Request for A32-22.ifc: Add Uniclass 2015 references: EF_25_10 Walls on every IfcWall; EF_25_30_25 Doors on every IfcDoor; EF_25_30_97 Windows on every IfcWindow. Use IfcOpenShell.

First a look at what the model holds.

```python
import ifcopenshell

model = ifcopenshell.open("A32-22.ifc")
print(model.schema)
print("classifications:", [c.Name for c in model.by_type("IfcClassification")])
for ifc_class in ("IfcDoor", "IfcRoof", "IfcStair", "IfcWall", "IfcWindow"):
    print(ifc_class, len(model.by_type(ifc_class)))
```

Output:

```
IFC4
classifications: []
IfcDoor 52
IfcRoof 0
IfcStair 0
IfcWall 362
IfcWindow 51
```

```python
import ifcopenshell
import ifcopenshell.api.classification

model = ifcopenshell.open("A32-22.ifc")

system = ifcopenshell.api.classification.add_classification(model, classification="Uniclass 2015")

codes = {
    "IfcWall": ("EF_25_10", "Walls"),
    "IfcDoor": ("EF_25_30_25", "Doors"),
    "IfcWindow": ("EF_25_30_97", "Windows"),
}
for ifc_class, (code, name) in codes.items():
    products = model.by_type(ifc_class)
    ifcopenshell.api.classification.add_reference(
        model, products=products, classification=system, identification=code, name=name
    )
    print(code, len(products))

model.write("A32-22_v2.ifc")
```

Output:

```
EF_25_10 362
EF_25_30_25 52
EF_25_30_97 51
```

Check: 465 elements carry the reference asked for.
